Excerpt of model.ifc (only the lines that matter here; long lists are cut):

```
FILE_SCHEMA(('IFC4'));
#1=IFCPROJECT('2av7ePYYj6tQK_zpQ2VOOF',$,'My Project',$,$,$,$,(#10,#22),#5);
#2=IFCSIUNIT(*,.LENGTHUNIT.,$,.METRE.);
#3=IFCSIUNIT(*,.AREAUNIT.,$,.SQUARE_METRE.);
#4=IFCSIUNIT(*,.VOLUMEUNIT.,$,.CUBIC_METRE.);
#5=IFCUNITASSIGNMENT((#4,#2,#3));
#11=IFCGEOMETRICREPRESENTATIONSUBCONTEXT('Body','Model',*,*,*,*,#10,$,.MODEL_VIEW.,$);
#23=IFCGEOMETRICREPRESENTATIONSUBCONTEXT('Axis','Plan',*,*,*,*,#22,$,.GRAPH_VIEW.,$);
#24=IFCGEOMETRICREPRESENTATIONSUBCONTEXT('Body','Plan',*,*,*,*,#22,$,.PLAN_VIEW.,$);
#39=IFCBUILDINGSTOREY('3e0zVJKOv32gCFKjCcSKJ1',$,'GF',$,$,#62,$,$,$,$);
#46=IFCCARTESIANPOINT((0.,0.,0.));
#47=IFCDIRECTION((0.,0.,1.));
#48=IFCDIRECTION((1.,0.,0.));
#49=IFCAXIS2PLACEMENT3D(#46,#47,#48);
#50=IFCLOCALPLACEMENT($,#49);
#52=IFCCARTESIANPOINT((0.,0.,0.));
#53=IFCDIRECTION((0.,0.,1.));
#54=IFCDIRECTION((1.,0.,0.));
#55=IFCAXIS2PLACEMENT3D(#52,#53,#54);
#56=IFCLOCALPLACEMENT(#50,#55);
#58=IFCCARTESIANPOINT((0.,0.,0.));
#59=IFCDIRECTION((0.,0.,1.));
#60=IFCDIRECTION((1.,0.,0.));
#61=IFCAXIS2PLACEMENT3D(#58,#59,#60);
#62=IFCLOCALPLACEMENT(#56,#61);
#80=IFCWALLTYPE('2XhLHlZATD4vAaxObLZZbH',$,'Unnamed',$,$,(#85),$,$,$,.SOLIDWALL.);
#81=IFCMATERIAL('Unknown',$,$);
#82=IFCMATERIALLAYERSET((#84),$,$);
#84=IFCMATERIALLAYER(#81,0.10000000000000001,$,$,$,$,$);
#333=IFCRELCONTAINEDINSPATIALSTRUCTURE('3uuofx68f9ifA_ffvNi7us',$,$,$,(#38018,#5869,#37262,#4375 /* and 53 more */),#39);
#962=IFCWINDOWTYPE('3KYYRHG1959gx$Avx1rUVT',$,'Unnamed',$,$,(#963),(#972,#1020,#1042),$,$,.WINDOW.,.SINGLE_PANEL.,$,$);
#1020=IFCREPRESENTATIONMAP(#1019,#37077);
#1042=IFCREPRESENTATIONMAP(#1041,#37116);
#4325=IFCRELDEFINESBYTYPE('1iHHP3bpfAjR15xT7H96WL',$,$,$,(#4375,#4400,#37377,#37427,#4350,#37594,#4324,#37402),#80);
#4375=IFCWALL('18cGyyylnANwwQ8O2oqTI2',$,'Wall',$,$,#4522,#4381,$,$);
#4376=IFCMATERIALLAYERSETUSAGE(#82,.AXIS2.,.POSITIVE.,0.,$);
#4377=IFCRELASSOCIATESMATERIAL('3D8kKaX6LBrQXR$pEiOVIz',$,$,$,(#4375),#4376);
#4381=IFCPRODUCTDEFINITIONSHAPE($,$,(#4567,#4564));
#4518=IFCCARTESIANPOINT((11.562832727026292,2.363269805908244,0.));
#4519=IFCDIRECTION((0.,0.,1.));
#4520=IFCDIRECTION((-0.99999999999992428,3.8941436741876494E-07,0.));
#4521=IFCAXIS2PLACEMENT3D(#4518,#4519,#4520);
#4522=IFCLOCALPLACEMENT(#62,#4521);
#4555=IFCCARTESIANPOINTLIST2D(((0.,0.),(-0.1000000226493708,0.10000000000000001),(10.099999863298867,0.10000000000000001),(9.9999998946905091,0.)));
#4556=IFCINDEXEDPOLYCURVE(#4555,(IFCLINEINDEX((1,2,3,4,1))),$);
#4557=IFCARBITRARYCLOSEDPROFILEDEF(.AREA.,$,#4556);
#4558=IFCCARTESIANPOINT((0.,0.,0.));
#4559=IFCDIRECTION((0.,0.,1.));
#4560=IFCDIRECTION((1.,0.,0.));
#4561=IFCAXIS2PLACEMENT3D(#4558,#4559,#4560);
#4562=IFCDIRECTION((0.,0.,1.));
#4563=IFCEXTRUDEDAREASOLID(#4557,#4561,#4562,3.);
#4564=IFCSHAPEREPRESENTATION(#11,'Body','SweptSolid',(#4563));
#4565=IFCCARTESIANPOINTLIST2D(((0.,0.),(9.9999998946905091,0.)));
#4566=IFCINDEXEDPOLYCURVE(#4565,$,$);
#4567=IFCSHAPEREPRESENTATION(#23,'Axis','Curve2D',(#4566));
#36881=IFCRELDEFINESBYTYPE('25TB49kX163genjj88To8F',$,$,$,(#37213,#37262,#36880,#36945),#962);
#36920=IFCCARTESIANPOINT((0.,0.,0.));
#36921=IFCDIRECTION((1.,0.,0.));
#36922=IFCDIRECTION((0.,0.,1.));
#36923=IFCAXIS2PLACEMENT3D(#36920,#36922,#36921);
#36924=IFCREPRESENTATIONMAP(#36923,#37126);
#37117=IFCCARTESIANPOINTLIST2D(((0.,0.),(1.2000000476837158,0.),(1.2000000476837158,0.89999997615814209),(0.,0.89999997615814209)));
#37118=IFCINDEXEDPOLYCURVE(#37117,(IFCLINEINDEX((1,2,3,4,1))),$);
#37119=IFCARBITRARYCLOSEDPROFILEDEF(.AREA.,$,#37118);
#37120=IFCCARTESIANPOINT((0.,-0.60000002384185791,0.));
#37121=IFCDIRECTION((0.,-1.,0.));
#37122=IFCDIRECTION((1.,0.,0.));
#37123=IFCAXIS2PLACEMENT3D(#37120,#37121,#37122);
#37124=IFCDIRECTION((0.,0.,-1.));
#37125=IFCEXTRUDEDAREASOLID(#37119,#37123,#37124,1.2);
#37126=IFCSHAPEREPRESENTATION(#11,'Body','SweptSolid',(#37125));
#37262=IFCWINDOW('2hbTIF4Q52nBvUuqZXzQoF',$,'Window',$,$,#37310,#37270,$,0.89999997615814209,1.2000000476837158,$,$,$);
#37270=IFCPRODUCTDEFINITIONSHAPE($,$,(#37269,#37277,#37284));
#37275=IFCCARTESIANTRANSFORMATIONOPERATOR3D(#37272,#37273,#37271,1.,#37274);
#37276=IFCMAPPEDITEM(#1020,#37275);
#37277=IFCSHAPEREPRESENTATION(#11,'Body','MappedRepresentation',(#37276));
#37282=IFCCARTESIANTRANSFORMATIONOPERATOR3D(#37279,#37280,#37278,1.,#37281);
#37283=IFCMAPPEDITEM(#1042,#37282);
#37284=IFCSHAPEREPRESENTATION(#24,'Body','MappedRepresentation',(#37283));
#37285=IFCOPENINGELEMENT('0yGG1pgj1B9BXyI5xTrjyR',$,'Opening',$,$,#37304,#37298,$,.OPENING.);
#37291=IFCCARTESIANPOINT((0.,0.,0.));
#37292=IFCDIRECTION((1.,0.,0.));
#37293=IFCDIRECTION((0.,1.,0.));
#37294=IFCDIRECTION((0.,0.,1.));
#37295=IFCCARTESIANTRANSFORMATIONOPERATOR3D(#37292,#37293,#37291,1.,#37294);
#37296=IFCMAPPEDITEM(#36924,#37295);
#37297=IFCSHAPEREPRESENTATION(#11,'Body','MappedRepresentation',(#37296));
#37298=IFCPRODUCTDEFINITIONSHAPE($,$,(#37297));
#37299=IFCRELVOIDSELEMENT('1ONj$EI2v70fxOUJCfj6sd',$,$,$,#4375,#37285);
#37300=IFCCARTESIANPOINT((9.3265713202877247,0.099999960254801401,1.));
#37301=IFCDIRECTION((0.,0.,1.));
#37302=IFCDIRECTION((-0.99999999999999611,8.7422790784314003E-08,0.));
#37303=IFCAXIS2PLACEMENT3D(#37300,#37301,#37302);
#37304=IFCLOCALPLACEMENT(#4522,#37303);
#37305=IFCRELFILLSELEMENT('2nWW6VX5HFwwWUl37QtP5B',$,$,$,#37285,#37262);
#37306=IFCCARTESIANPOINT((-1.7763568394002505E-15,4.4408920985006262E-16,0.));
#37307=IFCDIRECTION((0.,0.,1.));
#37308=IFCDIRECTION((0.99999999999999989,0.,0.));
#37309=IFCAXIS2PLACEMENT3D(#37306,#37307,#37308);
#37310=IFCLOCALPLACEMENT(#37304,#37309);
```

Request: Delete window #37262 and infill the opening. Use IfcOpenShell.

```python
import ifcopenshell
import ifcopenshell.api.feature
import ifcopenshell.api.root
import ifcopenshell.geom
import ifcopenshell.util.shape

model = ifcopenshell.open("model.ifc")
settings = ifcopenshell.geom.settings()


def volume(element):
    """Net volume in cubic metres, openings subtracted."""
    shape = ifcopenshell.geom.create_shape(settings, element)
    return ifcopenshell.util.shape.get_volume(shape.geometry)


window = model.by_guid("2hbTIF4Q52nBvUuqZXzQoF")
opening = window.FillsVoids[0].RelatingOpeningElement
wall = opening.VoidsElements[0].RelatingBuildingElement
before = volume(wall)

ifcopenshell.api.root.remove_product(model, product=window)
ifcopenshell.api.feature.remove_feature(model, feature=opening)

after = volume(wall)

print(f"wall volume {before:.3f} -> {after:.3f} m3")

model.write("model-out.ifc")
```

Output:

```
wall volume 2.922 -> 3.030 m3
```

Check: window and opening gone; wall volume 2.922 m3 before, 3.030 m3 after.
